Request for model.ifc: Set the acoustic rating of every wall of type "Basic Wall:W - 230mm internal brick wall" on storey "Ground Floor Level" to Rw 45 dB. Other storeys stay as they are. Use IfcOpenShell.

First a look at what the model holds.

```python
import ifcopenshell
import ifcopenshell.util.element

model = ifcopenshell.open("model.ifc")
print(model.schema)
storey = next(s for s in model.by_type("IfcBuildingStorey") if s.Name == "Ground Floor Level")
walls = [e for e in ifcopenshell.util.element.get_decomposition(storey) if e.is_a("IfcWall")]
seen = {}
for e in walls:
    element_type = ifcopenshell.util.element.get_type(e)
    key = (element_type.Name if element_type != e and element_type else None, ifcopenshell.util.element.get_pset(e, "Pset_WallCommon", "AcousticRating"))
    seen[key] = seen.get(key, 0) + 1
for (name, value), count in sorted(seen.items(), key=str):
    print(count, "x", name, "|", value)
```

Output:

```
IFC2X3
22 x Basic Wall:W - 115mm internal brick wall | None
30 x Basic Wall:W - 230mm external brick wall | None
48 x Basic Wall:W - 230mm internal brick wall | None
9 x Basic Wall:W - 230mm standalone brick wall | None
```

```python
import ifcopenshell
import ifcopenshell.api.pset
import ifcopenshell.util.element

model = ifcopenshell.open("model.ifc")

storey = next(s for s in model.by_type("IfcBuildingStorey") if s.Name == "Ground Floor Level")
walls = [e for e in ifcopenshell.util.element.get_decomposition(storey) if e.is_a("IfcWall")]

count = 0
for e in walls:
    element_type = ifcopenshell.util.element.get_type(e)
    if element_type in (None, e) or element_type.Name != "Basic Wall:W - 230mm internal brick wall":
        continue
    # add_pset returns the element's existing set when there is one.
    pset = ifcopenshell.api.pset.add_pset(model, product=e, name="Pset_WallCommon")
    ifcopenshell.api.pset.edit_pset(model, pset=pset, properties={"AcousticRating": "Rw 45 dB"})
    count += 1

print(count, "walls updated")

model.write("model_rev.ifc")
```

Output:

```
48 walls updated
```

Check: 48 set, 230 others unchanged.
